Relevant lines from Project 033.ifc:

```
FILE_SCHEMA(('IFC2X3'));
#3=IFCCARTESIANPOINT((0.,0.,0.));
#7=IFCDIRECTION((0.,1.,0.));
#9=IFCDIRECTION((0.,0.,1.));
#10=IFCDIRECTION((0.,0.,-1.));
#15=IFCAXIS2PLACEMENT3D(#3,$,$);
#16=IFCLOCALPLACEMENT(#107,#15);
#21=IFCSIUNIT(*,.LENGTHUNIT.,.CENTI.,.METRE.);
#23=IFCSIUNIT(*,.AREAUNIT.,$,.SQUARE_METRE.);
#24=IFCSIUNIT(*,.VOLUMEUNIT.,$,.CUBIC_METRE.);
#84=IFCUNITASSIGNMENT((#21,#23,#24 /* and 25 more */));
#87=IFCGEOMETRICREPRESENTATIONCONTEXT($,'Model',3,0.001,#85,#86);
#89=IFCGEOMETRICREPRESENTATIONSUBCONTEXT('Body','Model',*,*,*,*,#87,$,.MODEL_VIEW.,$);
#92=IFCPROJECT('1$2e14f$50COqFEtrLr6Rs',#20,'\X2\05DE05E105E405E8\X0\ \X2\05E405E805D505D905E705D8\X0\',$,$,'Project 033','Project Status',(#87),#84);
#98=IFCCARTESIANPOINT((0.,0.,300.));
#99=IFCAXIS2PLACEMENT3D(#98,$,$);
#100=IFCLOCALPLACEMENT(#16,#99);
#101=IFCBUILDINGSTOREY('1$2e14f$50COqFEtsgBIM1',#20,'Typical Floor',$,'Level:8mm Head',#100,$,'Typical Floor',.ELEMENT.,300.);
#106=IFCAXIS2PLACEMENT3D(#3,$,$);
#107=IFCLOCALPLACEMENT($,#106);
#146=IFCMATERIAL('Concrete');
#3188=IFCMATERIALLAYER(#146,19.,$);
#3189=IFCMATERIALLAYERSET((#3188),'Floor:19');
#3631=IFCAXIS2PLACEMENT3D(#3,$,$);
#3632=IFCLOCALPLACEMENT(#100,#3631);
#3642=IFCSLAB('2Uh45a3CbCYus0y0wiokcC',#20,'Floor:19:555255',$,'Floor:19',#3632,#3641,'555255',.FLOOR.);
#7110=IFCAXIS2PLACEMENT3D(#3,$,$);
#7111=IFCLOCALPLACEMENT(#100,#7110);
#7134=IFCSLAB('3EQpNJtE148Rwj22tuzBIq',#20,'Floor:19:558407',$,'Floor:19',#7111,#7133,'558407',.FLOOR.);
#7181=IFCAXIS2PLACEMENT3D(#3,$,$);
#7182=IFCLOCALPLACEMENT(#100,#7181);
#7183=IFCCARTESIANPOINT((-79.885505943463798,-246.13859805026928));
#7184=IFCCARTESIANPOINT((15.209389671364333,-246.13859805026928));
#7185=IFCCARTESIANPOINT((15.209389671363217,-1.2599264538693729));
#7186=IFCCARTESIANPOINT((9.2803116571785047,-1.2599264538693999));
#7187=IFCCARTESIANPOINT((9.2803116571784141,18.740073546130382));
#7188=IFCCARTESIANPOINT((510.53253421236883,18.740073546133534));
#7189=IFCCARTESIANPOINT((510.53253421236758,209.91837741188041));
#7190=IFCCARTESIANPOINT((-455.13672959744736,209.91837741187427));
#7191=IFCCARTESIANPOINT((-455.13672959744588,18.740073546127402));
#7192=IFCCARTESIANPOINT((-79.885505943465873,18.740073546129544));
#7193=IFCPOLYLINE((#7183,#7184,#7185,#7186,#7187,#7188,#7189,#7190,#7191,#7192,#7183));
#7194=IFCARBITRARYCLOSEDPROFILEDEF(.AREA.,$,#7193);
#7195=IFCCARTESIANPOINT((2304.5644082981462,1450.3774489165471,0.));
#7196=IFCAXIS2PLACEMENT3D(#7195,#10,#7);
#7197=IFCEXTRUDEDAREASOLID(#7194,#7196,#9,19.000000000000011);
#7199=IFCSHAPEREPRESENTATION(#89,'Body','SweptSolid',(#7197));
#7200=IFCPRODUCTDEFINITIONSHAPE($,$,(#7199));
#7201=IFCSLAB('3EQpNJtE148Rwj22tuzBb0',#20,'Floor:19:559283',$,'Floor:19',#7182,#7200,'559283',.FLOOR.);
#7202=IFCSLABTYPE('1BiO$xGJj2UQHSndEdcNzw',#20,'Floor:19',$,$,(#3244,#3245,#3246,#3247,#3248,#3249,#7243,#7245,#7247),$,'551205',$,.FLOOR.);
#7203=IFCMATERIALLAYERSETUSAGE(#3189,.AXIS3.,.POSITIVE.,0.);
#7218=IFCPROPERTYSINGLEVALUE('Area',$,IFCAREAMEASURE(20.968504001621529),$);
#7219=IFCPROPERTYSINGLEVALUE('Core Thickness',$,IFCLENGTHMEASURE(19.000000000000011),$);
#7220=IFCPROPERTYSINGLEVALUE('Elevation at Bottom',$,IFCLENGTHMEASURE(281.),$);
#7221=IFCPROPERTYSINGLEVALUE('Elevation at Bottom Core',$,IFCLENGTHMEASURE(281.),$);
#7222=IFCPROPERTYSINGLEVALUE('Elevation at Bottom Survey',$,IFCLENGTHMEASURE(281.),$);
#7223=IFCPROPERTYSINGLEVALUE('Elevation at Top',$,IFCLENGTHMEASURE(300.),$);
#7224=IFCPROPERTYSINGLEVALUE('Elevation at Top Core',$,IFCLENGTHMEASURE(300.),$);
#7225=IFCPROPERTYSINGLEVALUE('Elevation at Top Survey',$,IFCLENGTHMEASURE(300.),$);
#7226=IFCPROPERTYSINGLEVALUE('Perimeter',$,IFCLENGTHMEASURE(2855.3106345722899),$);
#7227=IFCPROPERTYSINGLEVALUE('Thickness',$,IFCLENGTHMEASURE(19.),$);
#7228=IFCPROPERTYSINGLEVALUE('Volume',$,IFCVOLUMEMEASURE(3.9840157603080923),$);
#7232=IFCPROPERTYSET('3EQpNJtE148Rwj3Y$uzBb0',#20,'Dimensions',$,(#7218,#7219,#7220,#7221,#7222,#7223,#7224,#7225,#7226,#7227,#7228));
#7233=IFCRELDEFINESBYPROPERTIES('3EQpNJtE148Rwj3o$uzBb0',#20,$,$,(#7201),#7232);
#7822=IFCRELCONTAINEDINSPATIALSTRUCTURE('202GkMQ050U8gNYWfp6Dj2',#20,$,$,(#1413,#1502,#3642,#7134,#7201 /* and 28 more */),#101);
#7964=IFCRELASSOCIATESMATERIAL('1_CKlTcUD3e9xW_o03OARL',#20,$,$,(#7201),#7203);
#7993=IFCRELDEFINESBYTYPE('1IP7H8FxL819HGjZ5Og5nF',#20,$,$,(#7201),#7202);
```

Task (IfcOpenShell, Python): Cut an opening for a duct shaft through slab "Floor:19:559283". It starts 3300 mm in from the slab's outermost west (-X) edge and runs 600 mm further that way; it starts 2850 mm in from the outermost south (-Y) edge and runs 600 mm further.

```python
import numpy as np
import ifcopenshell
import ifcopenshell.api.feature
import ifcopenshell.api.geometry
import ifcopenshell.api.pset
import ifcopenshell.api.root
import ifcopenshell.geom
import ifcopenshell.util.element
import ifcopenshell.util.placement
import ifcopenshell.util.representation
import ifcopenshell.util.shape
import ifcopenshell.util.unit

model = ifcopenshell.open("Project 033.ifc")
unit_scale = ifcopenshell.util.unit.calculate_unit_scale(model)
area_scale = ifcopenshell.util.unit.calculate_unit_scale(model, "AREAUNIT")
volume_scale = ifcopenshell.util.unit.calculate_unit_scale(model, "VOLUMEUNIT")
settings = ifcopenshell.geom.settings()


def volume(element):
    """Net volume in cubic metres, openings subtracted."""
    shape = ifcopenshell.geom.create_shape(settings, element)
    return ifcopenshell.util.shape.get_volume(shape.geometry)


slab = model.by_id(7201)
before = volume(slab)

# Extent in the slab's own axes, in metres. The edges named are its -X and -Y sides.
slab_shape = ifcopenshell.geom.create_shape(settings, slab)
vertices = ifcopenshell.util.shape.get_vertices(slab_shape.geometry)
x_min, y_min, bottom = vertices.min(axis=0)
top = vertices[:, 2].max()

opening = ifcopenshell.api.root.create_entity(model, ifc_class="IfcOpeningElement", name="Duct shaft opening")
context = ifcopenshell.util.representation.get_context(model, "Model", "Body", "MODEL_VIEW")
width, depth = 0.6, 0.6
outline = [(0.0, 0.0), (width, 0.0), (width, depth), (0.0, depth), (0.0, 0.0)]
# Overshoot both faces by 50 mm so the cut is clean.
shape = ifcopenshell.api.geometry.add_slab_representation(
    model, context=context, depth=top - bottom + 0.1, polyline=outline
)
ifcopenshell.api.geometry.assign_representation(model, product=opening, representation=shape)

matrix = ifcopenshell.util.placement.get_local_placement(slab.ObjectPlacement)
matrix[:, 3] = matrix @ np.append(np.array([x_min + 3.3, y_min + 2.85, bottom - 0.05]) / unit_scale, 1.0)
ifcopenshell.api.geometry.edit_object_placement(model, product=opening, matrix=matrix, is_si=False)
ifcopenshell.api.feature.add_feature(model, feature=opening, element=slab)

after = volume(slab)

# Update the slab's stored quantities.
pset = model.by_id(ifcopenshell.util.element.get_pset(slab, "Dimensions", should_inherit=False)["id"])
ifcopenshell.api.pset.edit_pset(model, pset=pset, properties={
    "Area": model.create_entity("IfcAreaMeasure", after / (top - bottom) / area_scale),
    "Volume": model.create_entity("IfcVolumeMeasure", after / volume_scale),
})

print(f"slab volume {before:.3f} -> {after:.3f} m3")

model.write("Project 033_v2.ifc")
```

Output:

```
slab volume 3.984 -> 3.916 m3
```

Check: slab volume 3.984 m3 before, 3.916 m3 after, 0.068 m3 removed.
